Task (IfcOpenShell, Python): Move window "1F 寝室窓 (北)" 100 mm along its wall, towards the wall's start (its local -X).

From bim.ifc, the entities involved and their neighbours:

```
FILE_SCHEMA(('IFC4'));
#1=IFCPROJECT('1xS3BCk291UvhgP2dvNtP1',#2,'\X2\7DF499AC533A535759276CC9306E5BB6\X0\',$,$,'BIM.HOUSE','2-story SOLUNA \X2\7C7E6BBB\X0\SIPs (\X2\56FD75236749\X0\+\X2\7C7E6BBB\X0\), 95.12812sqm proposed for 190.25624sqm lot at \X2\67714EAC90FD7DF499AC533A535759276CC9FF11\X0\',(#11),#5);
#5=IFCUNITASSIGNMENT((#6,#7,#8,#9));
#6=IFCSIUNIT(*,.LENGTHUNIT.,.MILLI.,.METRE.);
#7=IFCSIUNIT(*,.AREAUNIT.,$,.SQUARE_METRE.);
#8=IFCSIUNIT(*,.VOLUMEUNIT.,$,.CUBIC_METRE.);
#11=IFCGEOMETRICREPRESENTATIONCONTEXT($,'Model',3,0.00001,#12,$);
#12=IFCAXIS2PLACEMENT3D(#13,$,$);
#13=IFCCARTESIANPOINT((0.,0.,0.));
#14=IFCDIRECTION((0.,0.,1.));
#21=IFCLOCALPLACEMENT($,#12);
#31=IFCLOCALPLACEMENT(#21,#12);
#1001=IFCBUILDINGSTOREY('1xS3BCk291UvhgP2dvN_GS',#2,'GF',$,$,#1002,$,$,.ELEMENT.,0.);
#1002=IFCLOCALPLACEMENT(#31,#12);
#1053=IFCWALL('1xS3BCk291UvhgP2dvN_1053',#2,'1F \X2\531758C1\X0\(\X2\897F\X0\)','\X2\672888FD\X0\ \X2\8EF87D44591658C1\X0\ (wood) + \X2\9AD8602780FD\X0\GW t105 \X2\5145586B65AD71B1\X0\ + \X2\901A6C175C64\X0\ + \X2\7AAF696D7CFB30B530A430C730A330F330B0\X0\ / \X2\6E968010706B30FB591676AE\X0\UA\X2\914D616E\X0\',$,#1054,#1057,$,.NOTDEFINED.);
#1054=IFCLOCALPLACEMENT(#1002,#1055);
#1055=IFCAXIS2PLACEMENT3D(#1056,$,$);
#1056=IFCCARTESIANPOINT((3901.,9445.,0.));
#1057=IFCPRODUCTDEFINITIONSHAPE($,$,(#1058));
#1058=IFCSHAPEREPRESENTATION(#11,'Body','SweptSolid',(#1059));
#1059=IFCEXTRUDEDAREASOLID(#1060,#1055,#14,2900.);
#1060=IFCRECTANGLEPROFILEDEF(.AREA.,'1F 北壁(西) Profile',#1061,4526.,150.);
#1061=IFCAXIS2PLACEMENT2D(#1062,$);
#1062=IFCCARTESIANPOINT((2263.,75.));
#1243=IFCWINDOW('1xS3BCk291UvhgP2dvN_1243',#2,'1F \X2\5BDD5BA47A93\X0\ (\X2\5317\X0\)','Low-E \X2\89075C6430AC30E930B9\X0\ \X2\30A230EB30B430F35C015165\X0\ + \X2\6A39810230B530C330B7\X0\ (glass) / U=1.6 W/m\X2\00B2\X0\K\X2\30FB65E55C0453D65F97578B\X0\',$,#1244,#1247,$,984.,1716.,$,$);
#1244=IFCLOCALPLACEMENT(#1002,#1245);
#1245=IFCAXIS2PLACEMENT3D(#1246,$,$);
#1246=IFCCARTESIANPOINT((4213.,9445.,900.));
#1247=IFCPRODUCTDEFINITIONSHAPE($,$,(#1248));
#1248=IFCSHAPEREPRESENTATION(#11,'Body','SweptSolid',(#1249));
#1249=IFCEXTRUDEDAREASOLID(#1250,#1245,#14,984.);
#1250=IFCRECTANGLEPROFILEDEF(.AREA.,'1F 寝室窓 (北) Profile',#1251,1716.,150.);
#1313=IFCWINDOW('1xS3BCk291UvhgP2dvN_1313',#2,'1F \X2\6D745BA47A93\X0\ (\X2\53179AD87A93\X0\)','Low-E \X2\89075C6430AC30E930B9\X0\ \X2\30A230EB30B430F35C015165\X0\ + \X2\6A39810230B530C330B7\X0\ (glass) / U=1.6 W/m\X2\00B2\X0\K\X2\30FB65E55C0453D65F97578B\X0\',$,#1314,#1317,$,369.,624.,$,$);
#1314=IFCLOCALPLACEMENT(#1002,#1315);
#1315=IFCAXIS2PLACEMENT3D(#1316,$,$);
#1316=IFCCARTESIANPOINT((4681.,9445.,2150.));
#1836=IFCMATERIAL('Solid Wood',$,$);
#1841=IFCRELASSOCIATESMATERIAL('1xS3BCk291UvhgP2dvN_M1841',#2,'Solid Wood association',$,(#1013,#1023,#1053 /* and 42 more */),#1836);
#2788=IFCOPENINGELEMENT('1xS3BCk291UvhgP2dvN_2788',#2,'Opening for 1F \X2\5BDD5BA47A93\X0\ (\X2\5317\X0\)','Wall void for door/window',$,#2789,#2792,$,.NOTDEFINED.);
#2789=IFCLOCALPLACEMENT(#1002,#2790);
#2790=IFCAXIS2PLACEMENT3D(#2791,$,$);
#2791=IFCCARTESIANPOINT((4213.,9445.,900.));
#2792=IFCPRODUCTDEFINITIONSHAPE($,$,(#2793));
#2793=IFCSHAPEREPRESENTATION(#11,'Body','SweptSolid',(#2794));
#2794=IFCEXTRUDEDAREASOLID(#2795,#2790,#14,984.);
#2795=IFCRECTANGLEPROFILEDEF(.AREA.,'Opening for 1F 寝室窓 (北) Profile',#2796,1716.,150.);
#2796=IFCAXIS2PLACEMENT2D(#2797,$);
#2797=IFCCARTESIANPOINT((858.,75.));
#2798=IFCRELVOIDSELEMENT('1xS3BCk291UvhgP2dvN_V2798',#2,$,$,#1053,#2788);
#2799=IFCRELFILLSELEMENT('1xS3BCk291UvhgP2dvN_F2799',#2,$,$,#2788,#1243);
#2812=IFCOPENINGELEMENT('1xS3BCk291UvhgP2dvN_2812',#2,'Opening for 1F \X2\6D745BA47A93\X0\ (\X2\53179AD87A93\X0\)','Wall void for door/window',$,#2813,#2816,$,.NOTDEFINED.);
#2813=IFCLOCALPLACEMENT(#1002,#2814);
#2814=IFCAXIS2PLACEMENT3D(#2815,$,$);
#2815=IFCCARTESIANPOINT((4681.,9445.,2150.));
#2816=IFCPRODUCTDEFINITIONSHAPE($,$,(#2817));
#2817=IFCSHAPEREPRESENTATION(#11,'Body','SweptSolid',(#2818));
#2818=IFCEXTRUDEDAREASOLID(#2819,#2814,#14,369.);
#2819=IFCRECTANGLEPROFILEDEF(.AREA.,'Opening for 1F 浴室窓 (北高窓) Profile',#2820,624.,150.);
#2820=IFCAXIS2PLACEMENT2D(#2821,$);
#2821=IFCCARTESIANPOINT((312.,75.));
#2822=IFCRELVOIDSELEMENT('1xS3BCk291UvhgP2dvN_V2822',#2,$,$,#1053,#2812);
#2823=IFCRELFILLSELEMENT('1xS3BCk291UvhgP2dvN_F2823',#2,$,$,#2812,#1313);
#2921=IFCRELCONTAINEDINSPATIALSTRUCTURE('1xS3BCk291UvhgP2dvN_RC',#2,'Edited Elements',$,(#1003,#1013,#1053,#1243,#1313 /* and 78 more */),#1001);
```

```python
import ifcopenshell
import ifcopenshell.api.geometry
import ifcopenshell.util.placement

model = ifcopenshell.open("bim.ifc")

window = model.by_guid("1xS3BCk291UvhgP2dvN_1243")
opening = window.FillsVoids[0].RelatingOpeningElement
wall = opening.VoidsElements[0].RelatingBuildingElement

wall_matrix = ifcopenshell.util.placement.get_local_placement(wall.ObjectPlacement)
shift = wall_matrix[:3, 0] * -100.0
before = ifcopenshell.util.placement.get_local_placement(window.ObjectPlacement)[:3, 3].copy()

# The window is not placed relative to its opening, so move both.
for product in (opening, window):
    matrix = ifcopenshell.util.placement.get_local_placement(product.ObjectPlacement)
    matrix[:3, 3] += shift
    ifcopenshell.api.geometry.edit_object_placement(model, product=product, matrix=matrix, is_si=False)

after = ifcopenshell.util.placement.get_local_placement(window.ObjectPlacement)[:3, 3]
print("window moved by", (after - before).round(3) + 0.0)

model.write("bim_edited.ifc")
```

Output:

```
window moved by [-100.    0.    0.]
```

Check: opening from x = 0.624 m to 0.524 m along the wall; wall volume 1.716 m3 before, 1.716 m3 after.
